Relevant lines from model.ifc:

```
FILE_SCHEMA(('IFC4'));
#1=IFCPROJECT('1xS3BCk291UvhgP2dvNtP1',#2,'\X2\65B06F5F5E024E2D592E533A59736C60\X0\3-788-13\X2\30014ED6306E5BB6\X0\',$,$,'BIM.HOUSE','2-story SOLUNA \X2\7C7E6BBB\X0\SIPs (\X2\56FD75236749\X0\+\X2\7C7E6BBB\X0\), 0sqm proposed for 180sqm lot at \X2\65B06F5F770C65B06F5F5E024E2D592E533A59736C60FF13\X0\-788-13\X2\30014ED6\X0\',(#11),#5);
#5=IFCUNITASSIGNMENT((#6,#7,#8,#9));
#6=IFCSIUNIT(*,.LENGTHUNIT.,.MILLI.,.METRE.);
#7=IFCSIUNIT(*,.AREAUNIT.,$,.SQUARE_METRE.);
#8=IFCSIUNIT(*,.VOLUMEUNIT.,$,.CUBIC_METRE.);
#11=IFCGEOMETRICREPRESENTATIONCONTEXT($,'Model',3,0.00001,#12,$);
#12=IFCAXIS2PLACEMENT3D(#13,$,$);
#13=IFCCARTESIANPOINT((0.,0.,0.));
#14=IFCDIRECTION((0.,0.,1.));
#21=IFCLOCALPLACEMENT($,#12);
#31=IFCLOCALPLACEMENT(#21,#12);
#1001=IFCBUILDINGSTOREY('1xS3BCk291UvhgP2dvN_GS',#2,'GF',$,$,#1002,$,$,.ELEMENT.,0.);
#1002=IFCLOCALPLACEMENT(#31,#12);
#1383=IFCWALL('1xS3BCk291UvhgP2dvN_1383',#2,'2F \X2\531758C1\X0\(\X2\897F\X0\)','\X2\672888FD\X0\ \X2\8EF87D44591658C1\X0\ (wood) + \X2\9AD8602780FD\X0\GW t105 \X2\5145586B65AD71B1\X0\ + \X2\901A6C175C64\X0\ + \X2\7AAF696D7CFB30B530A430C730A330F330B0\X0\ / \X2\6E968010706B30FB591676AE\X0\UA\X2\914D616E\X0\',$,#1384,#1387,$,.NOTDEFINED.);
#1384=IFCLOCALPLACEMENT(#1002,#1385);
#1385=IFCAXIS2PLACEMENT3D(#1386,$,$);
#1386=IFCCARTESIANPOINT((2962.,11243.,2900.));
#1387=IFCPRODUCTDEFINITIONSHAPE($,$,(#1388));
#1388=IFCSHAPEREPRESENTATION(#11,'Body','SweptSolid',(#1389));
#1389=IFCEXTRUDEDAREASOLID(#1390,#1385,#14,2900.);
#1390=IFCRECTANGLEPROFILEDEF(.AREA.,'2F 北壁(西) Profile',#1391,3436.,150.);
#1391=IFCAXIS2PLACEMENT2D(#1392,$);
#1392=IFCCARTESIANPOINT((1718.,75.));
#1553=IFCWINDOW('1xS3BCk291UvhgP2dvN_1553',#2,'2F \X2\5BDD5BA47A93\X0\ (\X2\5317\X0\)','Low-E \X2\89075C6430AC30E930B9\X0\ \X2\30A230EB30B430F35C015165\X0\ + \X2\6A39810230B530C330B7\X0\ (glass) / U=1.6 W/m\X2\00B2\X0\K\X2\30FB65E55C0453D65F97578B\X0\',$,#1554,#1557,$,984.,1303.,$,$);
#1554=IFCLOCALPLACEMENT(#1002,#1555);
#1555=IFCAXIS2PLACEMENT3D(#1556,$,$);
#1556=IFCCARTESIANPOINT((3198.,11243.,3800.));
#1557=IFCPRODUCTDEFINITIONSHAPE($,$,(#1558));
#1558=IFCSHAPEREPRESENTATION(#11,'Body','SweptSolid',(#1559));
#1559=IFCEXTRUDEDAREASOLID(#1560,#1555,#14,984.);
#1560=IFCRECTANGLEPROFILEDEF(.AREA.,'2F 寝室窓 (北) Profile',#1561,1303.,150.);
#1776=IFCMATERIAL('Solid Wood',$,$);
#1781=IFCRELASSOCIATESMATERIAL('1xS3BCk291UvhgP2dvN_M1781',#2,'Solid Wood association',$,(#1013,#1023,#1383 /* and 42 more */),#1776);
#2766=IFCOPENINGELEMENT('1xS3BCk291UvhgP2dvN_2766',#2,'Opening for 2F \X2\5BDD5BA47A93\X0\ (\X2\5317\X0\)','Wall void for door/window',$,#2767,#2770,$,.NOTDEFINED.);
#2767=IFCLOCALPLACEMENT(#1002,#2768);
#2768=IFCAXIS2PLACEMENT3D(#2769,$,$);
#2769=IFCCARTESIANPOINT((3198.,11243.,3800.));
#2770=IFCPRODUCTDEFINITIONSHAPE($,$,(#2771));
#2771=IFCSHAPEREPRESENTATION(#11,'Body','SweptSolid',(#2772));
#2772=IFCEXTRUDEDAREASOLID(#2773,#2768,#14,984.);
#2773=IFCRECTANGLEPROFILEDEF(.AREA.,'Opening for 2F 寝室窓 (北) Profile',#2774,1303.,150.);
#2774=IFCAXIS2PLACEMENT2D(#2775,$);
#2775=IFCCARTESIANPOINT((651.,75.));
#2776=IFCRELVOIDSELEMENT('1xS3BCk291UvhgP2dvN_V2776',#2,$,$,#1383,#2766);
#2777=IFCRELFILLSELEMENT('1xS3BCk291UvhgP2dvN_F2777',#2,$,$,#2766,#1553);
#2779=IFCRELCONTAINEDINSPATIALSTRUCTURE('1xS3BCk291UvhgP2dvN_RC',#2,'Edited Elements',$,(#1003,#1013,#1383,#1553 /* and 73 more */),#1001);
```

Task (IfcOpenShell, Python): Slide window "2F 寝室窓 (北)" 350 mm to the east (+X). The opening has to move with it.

```python
import ifcopenshell
import ifcopenshell.api.geometry
import ifcopenshell.util.placement
import ifcopenshell.util.unit

model = ifcopenshell.open("model.ifc")
unit_scale = ifcopenshell.util.unit.calculate_unit_scale(model)

window = model.by_id(1553)
opening = window.FillsVoids[0].RelatingOpeningElement
wall = opening.VoidsElements[0].RelatingBuildingElement

wall_matrix = ifcopenshell.util.placement.get_local_placement(wall.ObjectPlacement)
shift = wall_matrix[:3, 0] * 0.35 / unit_scale
before = ifcopenshell.util.placement.get_local_placement(window.ObjectPlacement)[:3, 3].copy()

# The window is not placed relative to its opening, so move both.
for product in (opening, window):
    matrix = ifcopenshell.util.placement.get_local_placement(product.ObjectPlacement)
    matrix[:3, 3] += shift
    ifcopenshell.api.geometry.edit_object_placement(model, product=product, matrix=matrix, is_si=False)

after = ifcopenshell.util.placement.get_local_placement(window.ObjectPlacement)[:3, 3]
print("window moved by", (after - before).round(3) + 0.0)

model.write("model_edited.ifc")
```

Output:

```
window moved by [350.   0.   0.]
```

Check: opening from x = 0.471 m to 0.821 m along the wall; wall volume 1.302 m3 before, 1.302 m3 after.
